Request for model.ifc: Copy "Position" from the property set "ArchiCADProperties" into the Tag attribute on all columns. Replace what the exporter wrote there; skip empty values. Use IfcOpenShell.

First a look at what the model holds.

```python
import ifcopenshell
import ifcopenshell.util.element

model = ifcopenshell.open("model.ifc")
print(model.schema)
columns = model.by_type("IfcColumn")
print(len(columns), "columns")
for e in columns[:8]:
    source = ifcopenshell.util.element.get_pset(e, "ArchiCADProperties", "Position")
    target = e.Tag
    print(e.id(), repr(source), repr(target), sep=" | ")
```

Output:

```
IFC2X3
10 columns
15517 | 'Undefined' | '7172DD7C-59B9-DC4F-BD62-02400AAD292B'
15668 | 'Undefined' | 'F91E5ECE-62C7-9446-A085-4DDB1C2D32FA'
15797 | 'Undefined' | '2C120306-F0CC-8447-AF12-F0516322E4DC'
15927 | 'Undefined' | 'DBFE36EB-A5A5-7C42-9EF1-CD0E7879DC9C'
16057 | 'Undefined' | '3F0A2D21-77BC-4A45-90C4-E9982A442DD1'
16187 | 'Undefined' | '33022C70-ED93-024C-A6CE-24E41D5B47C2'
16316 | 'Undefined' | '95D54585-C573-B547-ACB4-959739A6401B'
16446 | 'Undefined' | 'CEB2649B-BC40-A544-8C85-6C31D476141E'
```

```python
import ifcopenshell
import ifcopenshell.util.element

model = ifcopenshell.open("model.ifc")

count = 0
for e in model.by_type("IfcColumn"):
    value = ifcopenshell.util.element.get_pset(e, "ArchiCADProperties", "Position")
    current = e.Tag
    if not value or not value.strip() or current == value:
        continue
    e.Tag = value
    count += 1

print(count, "columns updated")

model.write("model_rev.ifc")
```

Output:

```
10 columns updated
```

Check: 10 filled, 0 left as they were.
